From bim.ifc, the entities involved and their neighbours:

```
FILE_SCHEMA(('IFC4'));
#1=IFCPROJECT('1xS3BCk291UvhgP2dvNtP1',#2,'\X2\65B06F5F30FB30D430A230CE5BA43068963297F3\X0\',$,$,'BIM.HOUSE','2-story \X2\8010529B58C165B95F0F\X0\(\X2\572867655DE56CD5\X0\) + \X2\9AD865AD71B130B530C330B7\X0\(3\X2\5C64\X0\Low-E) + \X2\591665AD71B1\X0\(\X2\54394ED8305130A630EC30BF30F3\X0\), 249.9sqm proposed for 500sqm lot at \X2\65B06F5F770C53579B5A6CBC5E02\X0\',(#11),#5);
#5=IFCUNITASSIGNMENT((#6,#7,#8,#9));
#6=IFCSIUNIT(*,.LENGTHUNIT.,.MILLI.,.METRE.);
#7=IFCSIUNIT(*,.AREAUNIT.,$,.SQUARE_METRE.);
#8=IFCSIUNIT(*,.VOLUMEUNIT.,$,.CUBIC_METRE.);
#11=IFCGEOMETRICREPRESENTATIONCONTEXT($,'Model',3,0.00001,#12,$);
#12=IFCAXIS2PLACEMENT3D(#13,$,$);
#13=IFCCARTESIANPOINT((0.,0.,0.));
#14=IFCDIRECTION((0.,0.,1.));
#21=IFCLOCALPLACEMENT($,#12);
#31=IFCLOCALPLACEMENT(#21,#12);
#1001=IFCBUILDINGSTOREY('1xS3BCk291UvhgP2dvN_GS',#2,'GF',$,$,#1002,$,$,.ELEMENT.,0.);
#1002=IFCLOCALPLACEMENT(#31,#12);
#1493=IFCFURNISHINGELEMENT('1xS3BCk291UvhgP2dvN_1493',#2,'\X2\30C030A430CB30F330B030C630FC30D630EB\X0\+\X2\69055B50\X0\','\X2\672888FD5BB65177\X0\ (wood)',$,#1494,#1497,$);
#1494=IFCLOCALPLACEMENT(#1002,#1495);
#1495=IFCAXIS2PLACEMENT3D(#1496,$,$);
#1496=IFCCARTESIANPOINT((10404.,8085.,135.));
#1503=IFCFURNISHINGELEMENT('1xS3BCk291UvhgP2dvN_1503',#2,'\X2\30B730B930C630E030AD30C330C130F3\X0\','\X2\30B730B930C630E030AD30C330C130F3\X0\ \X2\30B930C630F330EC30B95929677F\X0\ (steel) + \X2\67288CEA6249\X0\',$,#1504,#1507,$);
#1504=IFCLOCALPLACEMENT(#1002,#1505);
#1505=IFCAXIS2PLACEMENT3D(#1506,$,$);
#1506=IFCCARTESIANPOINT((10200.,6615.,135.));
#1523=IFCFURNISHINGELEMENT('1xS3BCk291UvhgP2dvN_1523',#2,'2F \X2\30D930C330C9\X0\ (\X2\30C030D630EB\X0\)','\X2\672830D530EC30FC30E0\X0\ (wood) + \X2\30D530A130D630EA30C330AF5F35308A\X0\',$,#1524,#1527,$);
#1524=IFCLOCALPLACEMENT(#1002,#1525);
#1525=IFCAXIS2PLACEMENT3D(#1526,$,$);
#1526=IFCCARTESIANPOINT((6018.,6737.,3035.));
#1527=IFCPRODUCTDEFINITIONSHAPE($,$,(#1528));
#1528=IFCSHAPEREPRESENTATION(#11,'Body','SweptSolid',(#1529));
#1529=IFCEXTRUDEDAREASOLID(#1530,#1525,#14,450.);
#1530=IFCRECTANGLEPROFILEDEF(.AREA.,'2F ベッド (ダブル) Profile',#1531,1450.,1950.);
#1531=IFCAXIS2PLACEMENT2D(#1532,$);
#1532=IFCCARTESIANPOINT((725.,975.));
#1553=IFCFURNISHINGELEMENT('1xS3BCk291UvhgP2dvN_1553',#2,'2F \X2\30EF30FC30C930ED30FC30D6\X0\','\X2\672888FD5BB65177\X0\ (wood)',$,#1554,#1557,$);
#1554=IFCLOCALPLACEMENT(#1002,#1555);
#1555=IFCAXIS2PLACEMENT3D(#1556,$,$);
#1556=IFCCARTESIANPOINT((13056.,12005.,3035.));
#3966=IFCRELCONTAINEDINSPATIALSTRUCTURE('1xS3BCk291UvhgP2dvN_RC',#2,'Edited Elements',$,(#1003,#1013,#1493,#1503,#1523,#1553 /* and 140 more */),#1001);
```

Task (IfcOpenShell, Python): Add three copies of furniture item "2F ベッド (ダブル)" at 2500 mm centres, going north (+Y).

```python
import numpy as np
import ifcopenshell
import ifcopenshell.api.geometry
import ifcopenshell.api.root
import ifcopenshell.util.element
import ifcopenshell.util.placement

model = ifcopenshell.open("bim.ifc")


def reuse_history(source, copy):
    """copy_class also copies each property set's owner history, people and application; keep the originals."""
    for rel in copy.IsDefinedBy:
        if rel.is_a("IfcRelDefinesByProperties") and (history := rel.RelatingPropertyDefinition.OwnerHistory):
            rel.RelatingPropertyDefinition.OwnerHistory = source.OwnerHistory
            ifcopenshell.util.element.remove_deep2(model, history)


source = model.by_id(1523)
base = ifcopenshell.util.placement.get_local_placement(source.ObjectPlacement)
step = np.array([0.0, 1.0, 0.0]) * 2500.0

for i in range(1, 4):
    copy = ifcopenshell.api.root.copy_class(model, product=source)
    copy.Representation = ifcopenshell.util.element.copy_deep(
        model, source.Representation, exclude=["IfcGeometricRepresentationContext", "IfcRepresentationMap"]
    )
    reuse_history(source, copy)
    matrix = base.copy()
    matrix[:3, 3] += i * step
    print("added at", matrix[:3, 3].round(3) + 0.0)
    ifcopenshell.api.geometry.edit_object_placement(model, product=copy, matrix=matrix, is_si=False)

model.write("bim_updated.ifc")
```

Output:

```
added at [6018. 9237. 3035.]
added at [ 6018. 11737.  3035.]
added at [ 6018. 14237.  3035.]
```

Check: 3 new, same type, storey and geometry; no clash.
